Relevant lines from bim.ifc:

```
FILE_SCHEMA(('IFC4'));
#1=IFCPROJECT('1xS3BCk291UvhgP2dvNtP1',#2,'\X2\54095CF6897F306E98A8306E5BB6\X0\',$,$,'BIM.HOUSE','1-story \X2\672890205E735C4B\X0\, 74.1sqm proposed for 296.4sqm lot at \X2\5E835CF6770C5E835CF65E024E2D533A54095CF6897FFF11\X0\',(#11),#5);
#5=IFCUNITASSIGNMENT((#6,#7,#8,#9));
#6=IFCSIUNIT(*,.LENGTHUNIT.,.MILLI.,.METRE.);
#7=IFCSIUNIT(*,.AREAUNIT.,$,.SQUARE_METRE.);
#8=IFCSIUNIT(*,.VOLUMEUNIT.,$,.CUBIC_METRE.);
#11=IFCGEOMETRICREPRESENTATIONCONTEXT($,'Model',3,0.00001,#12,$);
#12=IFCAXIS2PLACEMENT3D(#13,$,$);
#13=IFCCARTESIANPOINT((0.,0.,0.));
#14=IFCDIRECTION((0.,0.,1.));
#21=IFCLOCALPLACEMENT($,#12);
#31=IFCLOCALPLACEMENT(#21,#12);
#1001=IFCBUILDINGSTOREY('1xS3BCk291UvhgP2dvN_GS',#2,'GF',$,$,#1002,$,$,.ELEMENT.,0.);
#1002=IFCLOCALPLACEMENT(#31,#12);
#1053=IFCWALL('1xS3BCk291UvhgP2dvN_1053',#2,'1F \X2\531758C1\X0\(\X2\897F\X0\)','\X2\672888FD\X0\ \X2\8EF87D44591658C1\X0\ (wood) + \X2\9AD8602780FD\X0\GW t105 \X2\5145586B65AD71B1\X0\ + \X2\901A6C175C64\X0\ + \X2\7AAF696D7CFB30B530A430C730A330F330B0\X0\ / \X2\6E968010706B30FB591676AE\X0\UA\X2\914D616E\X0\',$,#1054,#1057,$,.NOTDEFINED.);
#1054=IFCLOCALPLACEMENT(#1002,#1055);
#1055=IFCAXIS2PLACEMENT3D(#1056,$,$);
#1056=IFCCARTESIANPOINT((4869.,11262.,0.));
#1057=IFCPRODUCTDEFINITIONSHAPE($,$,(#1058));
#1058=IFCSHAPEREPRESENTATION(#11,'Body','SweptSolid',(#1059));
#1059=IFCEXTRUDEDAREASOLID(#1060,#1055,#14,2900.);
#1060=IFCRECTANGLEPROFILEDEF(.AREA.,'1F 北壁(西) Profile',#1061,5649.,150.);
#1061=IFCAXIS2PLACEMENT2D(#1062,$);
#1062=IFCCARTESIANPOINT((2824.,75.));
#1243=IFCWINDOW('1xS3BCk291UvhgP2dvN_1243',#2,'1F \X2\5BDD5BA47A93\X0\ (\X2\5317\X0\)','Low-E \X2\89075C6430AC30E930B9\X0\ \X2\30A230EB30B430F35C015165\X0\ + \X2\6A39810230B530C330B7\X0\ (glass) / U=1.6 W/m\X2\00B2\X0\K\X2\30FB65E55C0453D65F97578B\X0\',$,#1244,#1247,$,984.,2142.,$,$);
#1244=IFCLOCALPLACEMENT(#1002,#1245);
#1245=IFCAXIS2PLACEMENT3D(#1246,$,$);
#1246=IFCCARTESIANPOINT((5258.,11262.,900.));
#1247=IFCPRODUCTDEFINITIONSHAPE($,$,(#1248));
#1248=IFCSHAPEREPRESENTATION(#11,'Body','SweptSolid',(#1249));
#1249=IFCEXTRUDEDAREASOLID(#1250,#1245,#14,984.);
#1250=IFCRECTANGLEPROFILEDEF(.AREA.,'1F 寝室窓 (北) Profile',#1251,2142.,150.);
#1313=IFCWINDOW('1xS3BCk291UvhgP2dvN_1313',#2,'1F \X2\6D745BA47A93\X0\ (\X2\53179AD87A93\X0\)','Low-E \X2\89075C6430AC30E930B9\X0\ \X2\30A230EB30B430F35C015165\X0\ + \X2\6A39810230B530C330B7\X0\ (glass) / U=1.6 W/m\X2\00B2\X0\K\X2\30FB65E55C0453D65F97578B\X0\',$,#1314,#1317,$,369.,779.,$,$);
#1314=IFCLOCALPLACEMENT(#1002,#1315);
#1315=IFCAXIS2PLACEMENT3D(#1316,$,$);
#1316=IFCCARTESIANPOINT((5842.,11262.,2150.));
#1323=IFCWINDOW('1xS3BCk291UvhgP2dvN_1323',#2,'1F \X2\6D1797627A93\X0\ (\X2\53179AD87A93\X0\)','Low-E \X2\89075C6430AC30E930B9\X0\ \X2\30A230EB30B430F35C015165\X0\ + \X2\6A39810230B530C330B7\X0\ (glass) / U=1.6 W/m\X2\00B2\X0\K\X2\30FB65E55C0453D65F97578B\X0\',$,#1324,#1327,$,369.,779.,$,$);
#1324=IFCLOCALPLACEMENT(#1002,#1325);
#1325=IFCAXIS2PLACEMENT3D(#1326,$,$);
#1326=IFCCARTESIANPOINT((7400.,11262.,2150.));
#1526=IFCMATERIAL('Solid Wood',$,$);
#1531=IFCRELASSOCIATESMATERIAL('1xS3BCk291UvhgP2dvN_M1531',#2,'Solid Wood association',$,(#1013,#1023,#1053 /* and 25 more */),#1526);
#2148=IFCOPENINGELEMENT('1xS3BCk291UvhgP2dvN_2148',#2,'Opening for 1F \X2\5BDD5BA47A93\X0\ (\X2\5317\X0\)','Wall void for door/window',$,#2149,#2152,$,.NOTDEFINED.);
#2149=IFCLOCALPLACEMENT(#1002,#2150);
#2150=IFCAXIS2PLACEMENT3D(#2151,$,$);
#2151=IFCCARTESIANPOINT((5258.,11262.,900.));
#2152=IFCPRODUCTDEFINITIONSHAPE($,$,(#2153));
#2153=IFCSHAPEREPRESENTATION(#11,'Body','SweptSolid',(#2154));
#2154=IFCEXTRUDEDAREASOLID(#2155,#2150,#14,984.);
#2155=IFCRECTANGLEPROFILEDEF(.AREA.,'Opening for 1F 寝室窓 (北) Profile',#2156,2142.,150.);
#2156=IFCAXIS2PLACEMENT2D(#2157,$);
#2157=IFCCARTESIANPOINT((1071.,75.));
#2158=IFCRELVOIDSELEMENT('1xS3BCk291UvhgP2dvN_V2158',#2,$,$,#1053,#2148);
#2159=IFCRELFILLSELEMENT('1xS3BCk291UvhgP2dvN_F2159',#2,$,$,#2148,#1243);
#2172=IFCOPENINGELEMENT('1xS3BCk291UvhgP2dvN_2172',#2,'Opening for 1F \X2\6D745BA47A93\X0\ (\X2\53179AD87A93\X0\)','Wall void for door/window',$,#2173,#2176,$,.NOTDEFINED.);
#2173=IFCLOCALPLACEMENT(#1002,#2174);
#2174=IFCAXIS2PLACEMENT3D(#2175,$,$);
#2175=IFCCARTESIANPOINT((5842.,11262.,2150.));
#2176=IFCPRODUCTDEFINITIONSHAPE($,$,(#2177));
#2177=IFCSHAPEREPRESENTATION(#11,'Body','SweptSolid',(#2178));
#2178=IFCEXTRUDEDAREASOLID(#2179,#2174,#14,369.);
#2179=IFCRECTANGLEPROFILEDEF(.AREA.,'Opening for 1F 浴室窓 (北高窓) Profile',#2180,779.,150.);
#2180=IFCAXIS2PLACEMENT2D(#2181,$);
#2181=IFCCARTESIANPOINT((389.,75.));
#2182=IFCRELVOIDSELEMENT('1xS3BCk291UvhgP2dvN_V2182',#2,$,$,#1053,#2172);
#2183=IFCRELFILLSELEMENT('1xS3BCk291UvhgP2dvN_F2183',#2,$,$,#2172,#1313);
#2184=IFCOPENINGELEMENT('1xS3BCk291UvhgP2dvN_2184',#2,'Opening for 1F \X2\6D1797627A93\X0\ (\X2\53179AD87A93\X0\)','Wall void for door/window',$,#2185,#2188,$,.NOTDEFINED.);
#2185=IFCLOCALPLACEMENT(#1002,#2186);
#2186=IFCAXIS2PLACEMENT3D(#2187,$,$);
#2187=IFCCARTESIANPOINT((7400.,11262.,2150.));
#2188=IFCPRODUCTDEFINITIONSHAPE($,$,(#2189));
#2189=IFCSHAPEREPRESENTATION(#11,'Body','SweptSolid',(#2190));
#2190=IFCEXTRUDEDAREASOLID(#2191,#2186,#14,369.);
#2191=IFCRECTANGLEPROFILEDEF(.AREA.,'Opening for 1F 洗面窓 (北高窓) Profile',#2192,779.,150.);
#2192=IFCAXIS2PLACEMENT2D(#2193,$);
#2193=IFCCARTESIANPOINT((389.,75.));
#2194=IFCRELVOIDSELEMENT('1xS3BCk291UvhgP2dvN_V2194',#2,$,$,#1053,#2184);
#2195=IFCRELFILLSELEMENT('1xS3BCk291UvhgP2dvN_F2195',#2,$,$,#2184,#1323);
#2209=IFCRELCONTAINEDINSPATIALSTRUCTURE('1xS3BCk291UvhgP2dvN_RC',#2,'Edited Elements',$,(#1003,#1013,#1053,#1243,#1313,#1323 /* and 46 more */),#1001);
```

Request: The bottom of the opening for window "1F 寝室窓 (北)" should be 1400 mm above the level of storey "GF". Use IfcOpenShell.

```python
import numpy as np
import ifcopenshell
import ifcopenshell.api.geometry
import ifcopenshell.geom
import ifcopenshell.util.element
import ifcopenshell.util.placement
import ifcopenshell.util.shape
import ifcopenshell.util.unit

model = ifcopenshell.open("bim.ifc")
unit_scale = ifcopenshell.util.unit.calculate_unit_scale(model)

window = model.by_guid("1xS3BCk291UvhgP2dvN_1243")
opening = window.FillsVoids[0].RelatingOpeningElement
storey = ifcopenshell.util.element.get_container(window, ifc_class="IfcBuildingStorey")
level = ifcopenshell.util.placement.get_local_placement(storey.ObjectPlacement)[2, 3]

# The opening's origin need not be at the sill, so measure its lowest point.
shape = ifcopenshell.geom.create_shape(ifcopenshell.geom.settings(), opening)
bottom = ifcopenshell.util.shape.get_shape_bottom_elevation(shape, shape.geometry) / unit_scale
dz = level + 1400.0 - bottom

shift = np.array([0.0, 0.0, dz])
# The window is not placed relative to its opening, so move both.
for product in (opening, window):
    matrix = ifcopenshell.util.placement.get_local_placement(product.ObjectPlacement)
    matrix[:3, 3] += shift
    ifcopenshell.api.geometry.edit_object_placement(model, product=product, matrix=matrix, is_si=False)

print(f"moved by {dz * unit_scale:+.3f} m")

model.write("bim_v2.ifc")
```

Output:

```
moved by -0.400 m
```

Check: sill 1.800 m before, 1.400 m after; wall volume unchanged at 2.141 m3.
